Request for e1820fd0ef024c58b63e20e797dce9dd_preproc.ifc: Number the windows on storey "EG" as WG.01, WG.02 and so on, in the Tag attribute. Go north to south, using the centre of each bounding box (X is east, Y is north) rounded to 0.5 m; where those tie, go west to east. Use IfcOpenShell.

First a look at what the model holds.

```python
import ifcopenshell
import ifcopenshell.util.element
import ifcopenshell.util.placement

model = ifcopenshell.open("e1820fd0ef024c58b63e20e797dce9dd_preproc.ifc")
print(model.schema)
storey = next(s for s in model.by_type("IfcBuildingStorey") if s.Name == "EG")
windows = [e for e in ifcopenshell.util.element.get_decomposition(storey) if e.is_a("IfcWindow")]
for e in sorted(windows, key=lambda e: e.id()):
    origin = ifcopenshell.util.placement.get_local_placement(e.ObjectPlacement)[:3, 3]
    print(e.id(), e.Tag, e.Name, origin.round(2) + 0.0, sep=" | ")
```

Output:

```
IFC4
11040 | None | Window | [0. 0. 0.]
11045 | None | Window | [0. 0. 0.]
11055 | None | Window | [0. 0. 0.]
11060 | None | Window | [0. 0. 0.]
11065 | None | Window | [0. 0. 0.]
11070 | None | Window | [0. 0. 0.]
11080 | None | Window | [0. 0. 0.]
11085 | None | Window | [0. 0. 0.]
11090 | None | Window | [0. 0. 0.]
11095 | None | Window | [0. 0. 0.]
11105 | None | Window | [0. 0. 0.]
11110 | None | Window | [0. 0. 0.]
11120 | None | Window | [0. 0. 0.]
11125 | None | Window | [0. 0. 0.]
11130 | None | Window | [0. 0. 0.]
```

```python
import ifcopenshell
import ifcopenshell.geom
import ifcopenshell.util.element
import ifcopenshell.util.shape

model = ifcopenshell.open("e1820fd0ef024c58b63e20e797dce9dd_preproc.ifc")
settings = ifcopenshell.geom.settings()
settings.set("use-world-coords", True)


def centre(element):
    shape = ifcopenshell.geom.create_shape(settings, element)
    return ifcopenshell.util.shape.get_bbox_centroid(shape.geometry)


storey = next(s for s in model.by_type("IfcBuildingStorey") if s.Name == "EG")
windows = [e for e in ifcopenshell.util.element.get_decomposition(storey) if e.is_a("IfcWindow")]

# Insertion points can sit at a corner or the storey origin, so sort by the geometry (in metres).
centres = {e: centre(e) for e in windows}
windows.sort(key=lambda e: (-round(centres[e][1] / 0.5), centres[e][0]))

for i, e in enumerate(windows, start=1):
    number = f"WG.{i:02d}"
    e.Tag = number
    print(e.id(), number)

model.write("e1820fd0ef024c58b63e20e797dce9dd_preproc-out.ifc")
```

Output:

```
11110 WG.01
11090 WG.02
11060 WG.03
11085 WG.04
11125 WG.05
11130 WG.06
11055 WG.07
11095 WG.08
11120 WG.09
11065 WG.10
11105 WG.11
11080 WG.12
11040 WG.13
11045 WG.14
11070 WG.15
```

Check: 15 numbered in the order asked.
